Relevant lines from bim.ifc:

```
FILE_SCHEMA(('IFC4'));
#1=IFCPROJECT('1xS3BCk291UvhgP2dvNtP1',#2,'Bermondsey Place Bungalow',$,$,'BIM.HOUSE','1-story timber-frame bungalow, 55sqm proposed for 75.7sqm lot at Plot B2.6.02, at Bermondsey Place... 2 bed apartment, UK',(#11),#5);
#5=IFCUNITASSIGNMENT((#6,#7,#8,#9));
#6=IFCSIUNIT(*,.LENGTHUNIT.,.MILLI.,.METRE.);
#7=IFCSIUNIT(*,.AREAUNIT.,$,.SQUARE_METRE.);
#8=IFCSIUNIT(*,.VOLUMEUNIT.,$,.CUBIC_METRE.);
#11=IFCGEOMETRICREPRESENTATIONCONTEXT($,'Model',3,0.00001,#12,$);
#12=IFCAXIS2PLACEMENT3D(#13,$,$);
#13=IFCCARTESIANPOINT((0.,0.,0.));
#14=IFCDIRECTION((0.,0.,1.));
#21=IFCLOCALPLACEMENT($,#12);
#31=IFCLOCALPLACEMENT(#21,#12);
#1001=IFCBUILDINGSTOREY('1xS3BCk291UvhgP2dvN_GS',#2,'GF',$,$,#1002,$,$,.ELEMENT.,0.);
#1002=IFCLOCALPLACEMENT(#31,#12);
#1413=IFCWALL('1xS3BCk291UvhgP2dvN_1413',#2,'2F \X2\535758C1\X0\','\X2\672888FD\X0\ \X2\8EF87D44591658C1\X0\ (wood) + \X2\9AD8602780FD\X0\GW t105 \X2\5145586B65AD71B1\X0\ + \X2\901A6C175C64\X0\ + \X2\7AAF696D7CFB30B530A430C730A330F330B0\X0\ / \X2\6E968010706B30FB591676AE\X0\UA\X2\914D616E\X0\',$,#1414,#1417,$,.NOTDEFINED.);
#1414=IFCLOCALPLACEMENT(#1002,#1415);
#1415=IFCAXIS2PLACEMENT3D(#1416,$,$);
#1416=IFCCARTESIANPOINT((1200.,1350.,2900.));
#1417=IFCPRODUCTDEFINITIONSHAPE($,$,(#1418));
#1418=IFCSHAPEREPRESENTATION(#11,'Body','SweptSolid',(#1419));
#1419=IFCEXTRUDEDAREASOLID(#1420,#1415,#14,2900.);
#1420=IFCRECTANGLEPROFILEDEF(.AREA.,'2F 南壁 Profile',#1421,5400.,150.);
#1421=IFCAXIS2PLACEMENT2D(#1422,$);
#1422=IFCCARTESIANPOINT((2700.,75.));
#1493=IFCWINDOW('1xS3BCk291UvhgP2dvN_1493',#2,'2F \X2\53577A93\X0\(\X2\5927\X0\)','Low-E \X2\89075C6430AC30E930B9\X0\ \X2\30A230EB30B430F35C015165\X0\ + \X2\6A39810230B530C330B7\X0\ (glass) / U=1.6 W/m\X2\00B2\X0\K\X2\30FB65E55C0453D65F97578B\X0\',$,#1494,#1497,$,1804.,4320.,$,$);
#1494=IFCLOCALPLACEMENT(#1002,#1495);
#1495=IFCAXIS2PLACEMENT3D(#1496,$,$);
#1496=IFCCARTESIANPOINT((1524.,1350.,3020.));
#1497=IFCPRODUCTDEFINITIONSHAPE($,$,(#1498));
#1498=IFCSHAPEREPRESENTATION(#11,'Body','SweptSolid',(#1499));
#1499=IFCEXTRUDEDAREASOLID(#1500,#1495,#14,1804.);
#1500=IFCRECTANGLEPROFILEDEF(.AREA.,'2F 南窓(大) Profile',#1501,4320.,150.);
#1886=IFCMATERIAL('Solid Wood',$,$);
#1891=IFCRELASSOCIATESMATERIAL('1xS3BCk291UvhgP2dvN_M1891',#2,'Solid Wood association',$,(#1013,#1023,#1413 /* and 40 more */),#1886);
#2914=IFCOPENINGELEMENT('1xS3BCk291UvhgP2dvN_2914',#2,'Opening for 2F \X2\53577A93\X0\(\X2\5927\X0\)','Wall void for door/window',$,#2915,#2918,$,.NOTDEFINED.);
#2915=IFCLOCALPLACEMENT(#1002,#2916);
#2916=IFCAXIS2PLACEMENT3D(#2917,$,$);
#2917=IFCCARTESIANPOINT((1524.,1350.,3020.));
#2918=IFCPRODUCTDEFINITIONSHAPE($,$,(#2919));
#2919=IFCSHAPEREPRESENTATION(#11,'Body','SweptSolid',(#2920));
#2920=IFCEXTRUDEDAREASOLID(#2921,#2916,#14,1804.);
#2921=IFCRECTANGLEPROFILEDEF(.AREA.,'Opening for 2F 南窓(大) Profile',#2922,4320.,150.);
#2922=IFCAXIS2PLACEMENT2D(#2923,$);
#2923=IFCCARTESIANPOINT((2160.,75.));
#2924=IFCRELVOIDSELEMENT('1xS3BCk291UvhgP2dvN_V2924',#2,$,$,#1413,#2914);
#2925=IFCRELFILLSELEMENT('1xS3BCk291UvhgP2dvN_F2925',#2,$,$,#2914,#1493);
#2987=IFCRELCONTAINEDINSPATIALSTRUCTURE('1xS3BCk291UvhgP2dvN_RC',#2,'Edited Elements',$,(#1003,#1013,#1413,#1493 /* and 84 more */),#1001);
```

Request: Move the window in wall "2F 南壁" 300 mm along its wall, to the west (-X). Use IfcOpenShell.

```python
import ifcopenshell
import ifcopenshell.api.geometry
import ifcopenshell.util.placement
import ifcopenshell.util.unit

model = ifcopenshell.open("bim.ifc")
unit_scale = ifcopenshell.util.unit.calculate_unit_scale(model)

window = model.by_guid("1xS3BCk291UvhgP2dvN_1493")
opening = window.FillsVoids[0].RelatingOpeningElement
wall = opening.VoidsElements[0].RelatingBuildingElement

wall_matrix = ifcopenshell.util.placement.get_local_placement(wall.ObjectPlacement)
shift = wall_matrix[:3, 0] * -0.3 / unit_scale
before = ifcopenshell.util.placement.get_local_placement(window.ObjectPlacement)[:3, 3].copy()

# The window is not placed relative to its opening, so move both.
for product in (opening, window):
    matrix = ifcopenshell.util.placement.get_local_placement(product.ObjectPlacement)
    matrix[:3, 3] += shift
    ifcopenshell.api.geometry.edit_object_placement(model, product=product, matrix=matrix, is_si=False)

after = ifcopenshell.util.placement.get_local_placement(window.ObjectPlacement)[:3, 3]
print("window moved by", (after - before).round(3) + 0.0)

model.write("bim_updated.ifc")
```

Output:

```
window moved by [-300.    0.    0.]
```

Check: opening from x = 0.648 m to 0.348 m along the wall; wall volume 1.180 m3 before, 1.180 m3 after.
